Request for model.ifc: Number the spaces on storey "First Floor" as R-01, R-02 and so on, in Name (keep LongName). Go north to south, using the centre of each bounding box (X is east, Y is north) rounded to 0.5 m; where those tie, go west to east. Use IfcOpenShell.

First a look at what the model holds.

```python
import ifcopenshell
import ifcopenshell.util.element
import ifcopenshell.util.placement

model = ifcopenshell.open("model.ifc")
print(model.schema)
storey = next(s for s in model.by_type("IfcBuildingStorey") if s.Name == "First Floor")
spaces = [e for e in ifcopenshell.util.element.get_decomposition(storey) if e.is_a("IfcSpace")]
for e in sorted(spaces, key=lambda e: e.id()):
    origin = ifcopenshell.util.placement.get_local_placement(e.ObjectPlacement)[:3, 3]
    print(e.id(), e.Name, e.LongName, origin.round(2) + 0.0, sep=" | ")
```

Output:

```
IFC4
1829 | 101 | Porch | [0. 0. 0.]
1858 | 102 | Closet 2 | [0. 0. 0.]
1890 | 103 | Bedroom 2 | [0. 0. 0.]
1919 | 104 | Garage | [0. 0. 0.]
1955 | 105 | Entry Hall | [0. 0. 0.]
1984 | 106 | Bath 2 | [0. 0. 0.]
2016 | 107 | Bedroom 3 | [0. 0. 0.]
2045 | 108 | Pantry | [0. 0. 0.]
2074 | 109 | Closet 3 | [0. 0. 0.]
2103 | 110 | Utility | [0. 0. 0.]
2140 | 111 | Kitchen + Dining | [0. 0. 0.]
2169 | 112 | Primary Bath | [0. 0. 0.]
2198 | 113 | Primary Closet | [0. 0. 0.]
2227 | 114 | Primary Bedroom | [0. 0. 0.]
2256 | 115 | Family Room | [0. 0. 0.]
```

```python
import ifcopenshell
import ifcopenshell.geom
import ifcopenshell.util.element
import ifcopenshell.util.shape

model = ifcopenshell.open("model.ifc")
settings = ifcopenshell.geom.settings()
settings.set("use-world-coords", True)


def centre(element):
    shape = ifcopenshell.geom.create_shape(settings, element)
    return ifcopenshell.util.shape.get_bbox_centroid(shape.geometry)


storey = next(s for s in model.by_type("IfcBuildingStorey") if s.Name == "First Floor")
spaces = [e for e in ifcopenshell.util.element.get_decomposition(storey) if e.is_a("IfcSpace")]

# Insertion points can sit at a corner or the storey origin, so sort by the geometry (in metres).
centres = {e: centre(e) for e in spaces}
spaces.sort(key=lambda e: (-round(centres[e][1] / 0.5), centres[e][0]))

for i, e in enumerate(spaces, start=1):
    number = f"R-{i:02d}"
    e.Name = number
    print(e.id(), number)

model.write("model-out.ifc")
```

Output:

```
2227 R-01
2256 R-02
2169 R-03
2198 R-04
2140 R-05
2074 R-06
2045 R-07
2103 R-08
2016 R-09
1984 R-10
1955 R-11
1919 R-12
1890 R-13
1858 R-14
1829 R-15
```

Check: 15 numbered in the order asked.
